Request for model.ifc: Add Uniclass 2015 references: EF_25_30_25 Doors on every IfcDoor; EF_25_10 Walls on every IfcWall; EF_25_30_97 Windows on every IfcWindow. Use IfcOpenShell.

First a look at what the model holds.

```python
import ifcopenshell

model = ifcopenshell.open("model.ifc")
print(model.schema)
print("classifications:", [c.Name for c in model.by_type("IfcClassification")])
for ifc_class in ("IfcDoor", "IfcRoof", "IfcStair", "IfcWall", "IfcWindow"):
    print(ifc_class, len(model.by_type(ifc_class)))
```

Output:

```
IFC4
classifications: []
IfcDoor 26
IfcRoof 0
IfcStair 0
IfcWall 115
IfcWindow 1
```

```python
import ifcopenshell
import ifcopenshell.api.classification

model = ifcopenshell.open("model.ifc")

system = ifcopenshell.api.classification.add_classification(model, classification="Uniclass 2015")

codes = {
    "IfcDoor": ("EF_25_30_25", "Doors"),
    "IfcWall": ("EF_25_10", "Walls"),
    "IfcWindow": ("EF_25_30_97", "Windows"),
}
for ifc_class, (code, name) in codes.items():
    products = model.by_type(ifc_class)
    ifcopenshell.api.classification.add_reference(
        model, products=products, classification=system, identification=code, name=name
    )
    print(code, len(products))

model.write("model_v2.ifc")
```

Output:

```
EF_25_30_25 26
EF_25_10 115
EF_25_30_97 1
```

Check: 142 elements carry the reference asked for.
